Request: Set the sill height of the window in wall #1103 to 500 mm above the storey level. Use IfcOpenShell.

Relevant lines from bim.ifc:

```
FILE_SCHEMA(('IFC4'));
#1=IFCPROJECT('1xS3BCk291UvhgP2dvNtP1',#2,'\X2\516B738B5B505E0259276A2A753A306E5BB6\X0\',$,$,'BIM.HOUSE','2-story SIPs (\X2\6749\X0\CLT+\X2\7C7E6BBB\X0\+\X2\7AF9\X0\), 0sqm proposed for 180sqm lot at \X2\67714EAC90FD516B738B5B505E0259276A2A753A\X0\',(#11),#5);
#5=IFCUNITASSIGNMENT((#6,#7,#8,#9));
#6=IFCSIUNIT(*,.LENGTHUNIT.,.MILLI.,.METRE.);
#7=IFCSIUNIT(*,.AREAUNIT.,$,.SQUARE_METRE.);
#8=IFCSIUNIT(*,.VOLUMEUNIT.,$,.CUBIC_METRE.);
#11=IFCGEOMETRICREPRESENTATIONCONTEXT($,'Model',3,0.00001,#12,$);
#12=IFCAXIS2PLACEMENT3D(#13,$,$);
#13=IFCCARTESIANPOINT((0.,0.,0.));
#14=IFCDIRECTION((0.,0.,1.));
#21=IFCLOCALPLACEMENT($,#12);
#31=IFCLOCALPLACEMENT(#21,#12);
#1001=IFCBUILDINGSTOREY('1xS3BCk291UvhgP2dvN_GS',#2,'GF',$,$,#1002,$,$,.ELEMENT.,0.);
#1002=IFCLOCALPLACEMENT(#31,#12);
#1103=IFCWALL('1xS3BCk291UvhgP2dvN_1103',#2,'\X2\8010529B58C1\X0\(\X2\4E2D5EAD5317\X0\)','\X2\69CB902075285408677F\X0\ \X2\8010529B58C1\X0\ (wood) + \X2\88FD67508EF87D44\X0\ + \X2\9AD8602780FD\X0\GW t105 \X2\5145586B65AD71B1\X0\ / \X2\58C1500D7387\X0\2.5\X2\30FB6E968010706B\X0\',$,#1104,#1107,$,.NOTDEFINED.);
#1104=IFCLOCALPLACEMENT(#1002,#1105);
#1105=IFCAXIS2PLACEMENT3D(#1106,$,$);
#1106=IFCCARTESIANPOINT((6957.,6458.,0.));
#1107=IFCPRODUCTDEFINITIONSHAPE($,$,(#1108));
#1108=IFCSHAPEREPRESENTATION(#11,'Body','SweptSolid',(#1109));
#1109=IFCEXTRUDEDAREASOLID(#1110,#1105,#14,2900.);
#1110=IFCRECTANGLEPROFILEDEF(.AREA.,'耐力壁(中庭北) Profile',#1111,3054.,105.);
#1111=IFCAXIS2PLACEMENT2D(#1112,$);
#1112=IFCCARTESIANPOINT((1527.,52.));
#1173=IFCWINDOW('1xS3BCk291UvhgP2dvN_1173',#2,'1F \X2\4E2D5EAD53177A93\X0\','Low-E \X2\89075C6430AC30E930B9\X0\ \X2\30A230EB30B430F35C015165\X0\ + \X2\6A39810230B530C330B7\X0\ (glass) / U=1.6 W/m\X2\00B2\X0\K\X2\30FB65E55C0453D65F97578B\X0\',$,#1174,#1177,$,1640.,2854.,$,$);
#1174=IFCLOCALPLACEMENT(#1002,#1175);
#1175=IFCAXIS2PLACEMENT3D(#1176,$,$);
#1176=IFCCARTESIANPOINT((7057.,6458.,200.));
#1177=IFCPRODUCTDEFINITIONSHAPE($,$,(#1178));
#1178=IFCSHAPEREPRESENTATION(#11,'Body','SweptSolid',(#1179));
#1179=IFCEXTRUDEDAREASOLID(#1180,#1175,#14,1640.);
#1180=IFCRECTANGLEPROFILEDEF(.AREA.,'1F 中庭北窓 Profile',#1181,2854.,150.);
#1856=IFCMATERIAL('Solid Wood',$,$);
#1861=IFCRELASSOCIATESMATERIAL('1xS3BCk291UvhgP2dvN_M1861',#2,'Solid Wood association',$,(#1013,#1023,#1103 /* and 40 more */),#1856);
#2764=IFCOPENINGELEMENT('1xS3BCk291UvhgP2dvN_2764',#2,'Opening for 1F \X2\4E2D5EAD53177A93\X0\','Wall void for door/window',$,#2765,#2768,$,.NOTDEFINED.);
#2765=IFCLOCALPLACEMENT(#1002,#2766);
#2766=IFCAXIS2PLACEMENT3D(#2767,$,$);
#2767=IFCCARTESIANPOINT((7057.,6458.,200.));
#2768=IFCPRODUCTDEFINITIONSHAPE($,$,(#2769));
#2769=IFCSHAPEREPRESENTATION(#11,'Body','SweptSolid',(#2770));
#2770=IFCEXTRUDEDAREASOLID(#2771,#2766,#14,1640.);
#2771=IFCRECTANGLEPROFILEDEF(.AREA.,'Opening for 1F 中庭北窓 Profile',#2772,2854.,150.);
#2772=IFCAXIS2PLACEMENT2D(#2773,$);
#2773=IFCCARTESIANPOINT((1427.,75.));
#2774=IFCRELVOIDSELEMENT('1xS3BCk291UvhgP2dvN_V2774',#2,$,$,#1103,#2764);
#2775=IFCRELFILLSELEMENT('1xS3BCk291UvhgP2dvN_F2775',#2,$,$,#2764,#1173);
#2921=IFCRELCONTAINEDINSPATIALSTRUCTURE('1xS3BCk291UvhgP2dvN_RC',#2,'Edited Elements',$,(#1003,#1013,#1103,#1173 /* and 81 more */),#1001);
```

```python
import numpy as np
import ifcopenshell
import ifcopenshell.api.geometry
import ifcopenshell.geom
import ifcopenshell.util.element
import ifcopenshell.util.placement
import ifcopenshell.util.shape
import ifcopenshell.util.unit

model = ifcopenshell.open("bim.ifc")
unit_scale = ifcopenshell.util.unit.calculate_unit_scale(model)

window = model.by_guid("1xS3BCk291UvhgP2dvN_1173")
opening = window.FillsVoids[0].RelatingOpeningElement
storey = ifcopenshell.util.element.get_container(window, ifc_class="IfcBuildingStorey")
level = ifcopenshell.util.placement.get_local_placement(storey.ObjectPlacement)[2, 3]

# The opening's origin need not be at the sill, so measure its lowest point.
shape = ifcopenshell.geom.create_shape(ifcopenshell.geom.settings(), opening)
bottom = ifcopenshell.util.shape.get_shape_bottom_elevation(shape, shape.geometry) / unit_scale
dz = level + 500.0 - bottom

shift = np.array([0.0, 0.0, dz])
# The window is not placed relative to its opening, so move both.
for product in (opening, window):
    matrix = ifcopenshell.util.placement.get_local_placement(product.ObjectPlacement)
    matrix[:3, 3] += shift
    ifcopenshell.api.geometry.edit_object_placement(model, product=product, matrix=matrix, is_si=False)

print(f"moved by {dz * unit_scale:+.3f} m")

model.write("bim_rev.ifc")
```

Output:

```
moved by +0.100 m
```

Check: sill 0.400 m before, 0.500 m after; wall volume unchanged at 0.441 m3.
